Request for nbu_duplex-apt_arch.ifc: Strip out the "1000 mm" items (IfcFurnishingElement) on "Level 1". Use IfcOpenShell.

First a look at what the model holds.

```python
import ifcopenshell
import ifcopenshell.util.element

model = ifcopenshell.open("nbu_duplex-apt_arch.ifc")
print(model.schema)
storey = next(s for s in model.by_type("IfcBuildingStorey") if s.Name == "Level 1")
furniture = [e for e in ifcopenshell.util.element.get_decomposition(storey) if e.is_a("IfcFurnishingElement")]
seen = {}
for e in furniture:
    element_type = ifcopenshell.util.element.get_type(e)
    name = element_type.Name if element_type not in (None, e) else None
    seen[name] = seen.get(name, 0) + 1
for name, count in sorted(seen.items(), key=str):
    print(count, "x", name)
```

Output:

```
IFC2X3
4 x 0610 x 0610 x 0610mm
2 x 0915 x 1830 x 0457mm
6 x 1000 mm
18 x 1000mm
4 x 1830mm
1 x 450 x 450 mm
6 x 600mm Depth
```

```python
import ifcopenshell
import ifcopenshell.api.root
import ifcopenshell.util.element

model = ifcopenshell.open("nbu_duplex-apt_arch.ifc")

storey = next(s for s in model.by_type("IfcBuildingStorey") if s.Name == "Level 1")
furniture = [e for e in ifcopenshell.util.element.get_decomposition(storey) if e.is_a("IfcFurnishingElement")]
targets = [e for e in furniture if (t := ifcopenshell.util.element.get_type(e)) not in (None, e) and t.Name == "1000 mm"]

for e in targets:
    ifcopenshell.api.root.remove_product(model, product=e)
print(len(targets), "removed")

model.write("nbu_duplex-apt_arch_rev.ifc")
```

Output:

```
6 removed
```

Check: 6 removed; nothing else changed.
